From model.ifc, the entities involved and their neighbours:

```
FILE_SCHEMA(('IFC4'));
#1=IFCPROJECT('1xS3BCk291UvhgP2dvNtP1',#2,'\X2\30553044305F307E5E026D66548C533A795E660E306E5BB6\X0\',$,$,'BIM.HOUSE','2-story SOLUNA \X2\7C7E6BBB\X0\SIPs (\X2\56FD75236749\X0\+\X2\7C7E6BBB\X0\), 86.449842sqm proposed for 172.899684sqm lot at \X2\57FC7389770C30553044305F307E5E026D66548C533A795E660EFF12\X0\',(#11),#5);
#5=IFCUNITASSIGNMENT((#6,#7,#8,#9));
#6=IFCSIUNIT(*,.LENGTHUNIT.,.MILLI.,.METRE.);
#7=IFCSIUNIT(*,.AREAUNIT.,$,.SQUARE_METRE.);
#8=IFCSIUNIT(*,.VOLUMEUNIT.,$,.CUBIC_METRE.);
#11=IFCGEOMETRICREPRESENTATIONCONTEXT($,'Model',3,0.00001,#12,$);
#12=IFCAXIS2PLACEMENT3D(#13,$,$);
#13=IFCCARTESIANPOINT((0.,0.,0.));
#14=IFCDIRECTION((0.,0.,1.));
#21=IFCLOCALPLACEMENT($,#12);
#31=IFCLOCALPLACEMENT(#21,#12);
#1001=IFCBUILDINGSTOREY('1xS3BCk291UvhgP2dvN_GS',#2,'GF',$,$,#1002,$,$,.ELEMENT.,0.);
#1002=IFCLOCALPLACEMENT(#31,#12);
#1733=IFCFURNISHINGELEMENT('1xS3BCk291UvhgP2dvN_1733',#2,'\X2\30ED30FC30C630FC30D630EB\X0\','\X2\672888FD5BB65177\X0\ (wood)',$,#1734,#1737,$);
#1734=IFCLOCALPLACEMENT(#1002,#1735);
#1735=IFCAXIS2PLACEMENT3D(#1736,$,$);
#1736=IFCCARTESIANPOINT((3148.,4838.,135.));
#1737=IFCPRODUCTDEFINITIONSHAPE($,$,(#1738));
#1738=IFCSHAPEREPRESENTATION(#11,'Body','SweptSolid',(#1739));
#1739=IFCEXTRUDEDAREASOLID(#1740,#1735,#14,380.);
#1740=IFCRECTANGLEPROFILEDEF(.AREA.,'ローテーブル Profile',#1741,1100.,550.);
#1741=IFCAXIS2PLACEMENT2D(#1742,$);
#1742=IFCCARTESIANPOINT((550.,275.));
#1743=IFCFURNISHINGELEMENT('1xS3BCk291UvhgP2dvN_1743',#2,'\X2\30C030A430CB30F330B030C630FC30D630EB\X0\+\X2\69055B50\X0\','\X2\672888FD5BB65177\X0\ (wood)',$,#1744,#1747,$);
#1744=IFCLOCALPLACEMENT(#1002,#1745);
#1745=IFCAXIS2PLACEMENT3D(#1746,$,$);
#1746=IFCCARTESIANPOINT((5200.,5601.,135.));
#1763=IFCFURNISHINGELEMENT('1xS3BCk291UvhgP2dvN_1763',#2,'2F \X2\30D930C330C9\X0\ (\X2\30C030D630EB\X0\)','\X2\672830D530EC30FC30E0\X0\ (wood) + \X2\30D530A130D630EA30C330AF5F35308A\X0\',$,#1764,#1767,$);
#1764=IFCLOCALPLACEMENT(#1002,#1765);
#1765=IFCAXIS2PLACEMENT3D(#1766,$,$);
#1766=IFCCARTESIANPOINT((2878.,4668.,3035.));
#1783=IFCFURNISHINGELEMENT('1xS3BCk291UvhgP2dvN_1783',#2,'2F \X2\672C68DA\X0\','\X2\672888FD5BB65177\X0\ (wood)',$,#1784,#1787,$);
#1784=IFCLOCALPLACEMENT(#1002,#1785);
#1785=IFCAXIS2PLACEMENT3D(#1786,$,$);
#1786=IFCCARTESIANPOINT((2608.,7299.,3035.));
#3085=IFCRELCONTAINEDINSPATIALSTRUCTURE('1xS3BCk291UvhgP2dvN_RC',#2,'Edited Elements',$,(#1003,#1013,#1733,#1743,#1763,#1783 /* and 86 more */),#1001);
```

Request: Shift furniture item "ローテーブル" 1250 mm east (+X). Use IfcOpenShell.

```python
import ifcopenshell
import ifcopenshell.api.geometry
import ifcopenshell.util.placement
import ifcopenshell.util.unit

model = ifcopenshell.open("model.ifc")
unit_scale = ifcopenshell.util.unit.calculate_unit_scale(model)

item = model.by_guid("1xS3BCk291UvhgP2dvN_1733")
matrix = ifcopenshell.util.placement.get_local_placement(item.ObjectPlacement)
matrix[0, 3] += 1.25 / unit_scale
ifcopenshell.api.geometry.edit_object_placement(model, product=item, matrix=matrix, is_si=False)

print(ifcopenshell.util.placement.get_local_placement(item.ObjectPlacement).round(3) + 0.0)

model.write("model-out.ifc")
```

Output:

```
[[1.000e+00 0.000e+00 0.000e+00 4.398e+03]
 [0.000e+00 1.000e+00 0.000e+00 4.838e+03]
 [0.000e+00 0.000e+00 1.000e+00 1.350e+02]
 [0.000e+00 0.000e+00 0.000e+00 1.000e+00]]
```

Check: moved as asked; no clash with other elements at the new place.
